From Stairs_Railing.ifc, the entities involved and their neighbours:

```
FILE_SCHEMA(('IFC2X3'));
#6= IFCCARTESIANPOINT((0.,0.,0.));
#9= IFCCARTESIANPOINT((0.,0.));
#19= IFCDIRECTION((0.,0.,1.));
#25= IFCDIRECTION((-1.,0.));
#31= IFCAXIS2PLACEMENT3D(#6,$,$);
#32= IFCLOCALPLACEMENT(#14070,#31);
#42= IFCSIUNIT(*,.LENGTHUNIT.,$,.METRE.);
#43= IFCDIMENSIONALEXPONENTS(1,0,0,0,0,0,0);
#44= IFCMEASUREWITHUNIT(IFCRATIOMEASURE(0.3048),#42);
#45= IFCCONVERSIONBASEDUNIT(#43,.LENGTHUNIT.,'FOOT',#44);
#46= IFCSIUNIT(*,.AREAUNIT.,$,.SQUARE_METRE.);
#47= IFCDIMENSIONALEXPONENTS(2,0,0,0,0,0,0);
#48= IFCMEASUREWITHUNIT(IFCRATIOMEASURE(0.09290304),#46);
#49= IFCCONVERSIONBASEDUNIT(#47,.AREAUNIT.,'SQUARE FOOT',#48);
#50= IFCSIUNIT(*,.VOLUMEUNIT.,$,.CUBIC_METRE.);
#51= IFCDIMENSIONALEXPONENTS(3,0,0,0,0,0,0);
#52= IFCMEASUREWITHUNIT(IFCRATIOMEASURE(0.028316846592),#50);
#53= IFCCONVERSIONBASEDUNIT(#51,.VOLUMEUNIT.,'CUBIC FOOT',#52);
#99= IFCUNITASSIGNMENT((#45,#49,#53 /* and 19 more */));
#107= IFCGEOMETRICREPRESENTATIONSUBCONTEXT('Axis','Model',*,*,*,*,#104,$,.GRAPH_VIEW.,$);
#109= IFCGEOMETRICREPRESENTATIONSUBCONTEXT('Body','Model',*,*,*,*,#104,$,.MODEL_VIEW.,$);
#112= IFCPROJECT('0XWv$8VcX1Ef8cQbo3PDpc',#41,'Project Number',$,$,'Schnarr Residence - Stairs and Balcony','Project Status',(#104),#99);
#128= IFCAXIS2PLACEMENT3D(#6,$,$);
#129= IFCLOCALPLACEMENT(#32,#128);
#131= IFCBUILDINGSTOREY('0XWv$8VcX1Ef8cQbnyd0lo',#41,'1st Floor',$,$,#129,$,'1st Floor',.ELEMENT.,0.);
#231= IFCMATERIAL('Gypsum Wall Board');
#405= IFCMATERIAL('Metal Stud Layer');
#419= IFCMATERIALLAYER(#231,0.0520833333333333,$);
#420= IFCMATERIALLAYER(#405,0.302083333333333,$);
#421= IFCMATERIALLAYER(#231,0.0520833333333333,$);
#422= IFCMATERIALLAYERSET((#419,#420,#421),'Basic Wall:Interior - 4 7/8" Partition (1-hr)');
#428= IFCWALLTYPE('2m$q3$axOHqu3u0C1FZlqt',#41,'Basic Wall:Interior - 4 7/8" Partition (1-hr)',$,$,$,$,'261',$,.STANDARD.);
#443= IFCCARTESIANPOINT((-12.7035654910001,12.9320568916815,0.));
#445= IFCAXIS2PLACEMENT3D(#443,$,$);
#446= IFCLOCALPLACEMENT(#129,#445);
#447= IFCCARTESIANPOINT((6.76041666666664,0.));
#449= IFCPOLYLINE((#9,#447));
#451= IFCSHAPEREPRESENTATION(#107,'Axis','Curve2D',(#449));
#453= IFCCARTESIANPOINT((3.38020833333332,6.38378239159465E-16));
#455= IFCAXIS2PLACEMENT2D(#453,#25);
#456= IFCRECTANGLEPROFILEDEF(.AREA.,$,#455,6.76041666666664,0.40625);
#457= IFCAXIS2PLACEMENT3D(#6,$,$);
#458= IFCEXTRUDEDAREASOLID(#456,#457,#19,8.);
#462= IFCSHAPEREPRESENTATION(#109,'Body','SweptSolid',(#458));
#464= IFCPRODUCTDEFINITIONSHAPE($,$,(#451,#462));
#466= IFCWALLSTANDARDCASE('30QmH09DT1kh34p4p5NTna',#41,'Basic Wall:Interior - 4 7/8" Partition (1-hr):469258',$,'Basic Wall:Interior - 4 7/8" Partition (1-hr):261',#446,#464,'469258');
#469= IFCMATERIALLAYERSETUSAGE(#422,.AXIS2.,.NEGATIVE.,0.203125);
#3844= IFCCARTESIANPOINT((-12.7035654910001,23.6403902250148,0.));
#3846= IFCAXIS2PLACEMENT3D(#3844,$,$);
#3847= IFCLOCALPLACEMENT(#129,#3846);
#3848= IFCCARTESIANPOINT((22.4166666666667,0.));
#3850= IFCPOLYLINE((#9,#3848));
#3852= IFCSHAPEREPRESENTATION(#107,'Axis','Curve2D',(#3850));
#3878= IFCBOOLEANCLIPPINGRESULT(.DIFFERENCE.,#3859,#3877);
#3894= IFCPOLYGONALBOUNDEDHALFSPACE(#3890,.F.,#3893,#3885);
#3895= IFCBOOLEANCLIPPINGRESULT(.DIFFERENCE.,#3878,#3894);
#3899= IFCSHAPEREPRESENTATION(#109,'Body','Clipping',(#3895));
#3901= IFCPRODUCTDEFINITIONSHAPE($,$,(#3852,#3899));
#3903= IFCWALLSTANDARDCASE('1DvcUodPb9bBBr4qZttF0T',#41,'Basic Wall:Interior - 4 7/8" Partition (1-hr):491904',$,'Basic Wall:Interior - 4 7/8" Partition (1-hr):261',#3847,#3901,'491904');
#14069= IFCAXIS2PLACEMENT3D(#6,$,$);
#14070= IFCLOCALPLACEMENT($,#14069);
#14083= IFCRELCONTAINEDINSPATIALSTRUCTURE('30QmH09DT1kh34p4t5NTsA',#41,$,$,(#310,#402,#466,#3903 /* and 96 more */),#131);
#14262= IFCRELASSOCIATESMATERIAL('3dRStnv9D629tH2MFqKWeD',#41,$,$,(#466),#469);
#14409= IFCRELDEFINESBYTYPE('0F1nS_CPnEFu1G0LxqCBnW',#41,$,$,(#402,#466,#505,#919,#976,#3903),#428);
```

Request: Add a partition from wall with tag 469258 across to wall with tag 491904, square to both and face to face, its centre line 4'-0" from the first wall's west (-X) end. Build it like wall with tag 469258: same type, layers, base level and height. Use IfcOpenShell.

```python
import numpy as np
import ifcopenshell
import ifcopenshell.api.geometry
import ifcopenshell.api.material
import ifcopenshell.api.pset
import ifcopenshell.api.root
import ifcopenshell.api.spatial
import ifcopenshell.api.type
import ifcopenshell.geom
import ifcopenshell.util.element
import ifcopenshell.util.placement
import ifcopenshell.util.representation
import ifcopenshell.util.shape
import ifcopenshell.util.unit

model = ifcopenshell.open("Stairs_Railing.ifc")
unit_scale = ifcopenshell.util.unit.calculate_unit_scale(model)
settings = ifcopenshell.geom.settings()
settings.set("use-world-coords", True)

start_wall = model.by_guid("30QmH09DT1kh34p4p5NTna")
end_wall = model.by_guid("1DvcUodPb9bBBr4qZttF0T")
like = model.by_id(466)
matrix = ifcopenshell.util.placement.get_local_placement(start_wall.ObjectPlacement)
matrix[:3, 3] *= unit_scale


def extent(element):
    """Bounding box in the first wall's axes, in metres."""
    shape = ifcopenshell.geom.create_shape(settings, element)
    points = (ifcopenshell.util.shape.get_vertices(shape.geometry) - matrix[:3, 3]) @ matrix[:3, :3]
    return points.min(axis=0), points.max(axis=0)


y_start = extent(start_wall)[1][1]
y_end = extent(end_wall)[0][1]
like_min, like_max = extent(like)
length, height = float(abs(y_end - y_start)), float(like_max[2] - like_min[2])
layer_set = ifcopenshell.util.element.get_material(like, should_skip_usage=True)
thickness = sum(layer.LayerThickness for layer in layer_set.MaterialLayers) * unit_scale

wall = ifcopenshell.api.root.create_entity(model, ifc_class="IfcWallStandardCase", name="New partition")
storey = ifcopenshell.util.element.get_container(like)
ifcopenshell.api.spatial.assign_container(model, products=[wall], relating_structure=storey)
ifcopenshell.api.type.assign_type(
    model, related_objects=[wall], relating_type=ifcopenshell.util.element.get_type(like), should_map_representations=False
)
rel = ifcopenshell.api.material.assign_material(
    model, products=[wall], type="IfcMaterialLayerSetUsage", material=layer_set
)
rel.RelatingMaterial.OffsetFromReferenceLine = -thickness / 2 / unit_scale
pset = ifcopenshell.api.pset.add_pset(model, product=wall, name="Pset_WallCommon")
ifcopenshell.api.pset.edit_pset(model, pset=pset, properties={"IsExternal": False, "LoadBearing": False})

# The axis runs down the middle of the wall.
axis = ifcopenshell.api.geometry.add_axis_representation(
    model, context=ifcopenshell.util.representation.get_context(model, "Model", "Axis"), axis=[(0.0, 0.0), (length, 0.0)]
)
body = ifcopenshell.api.geometry.add_wall_representation(
    model,
    context=ifcopenshell.util.representation.get_context(model, "Model", "Body", "MODEL_VIEW"),
    length=length,
    height=height,
    thickness=thickness,
    offset=-thickness / 2,
)
for representation in (axis, body):
    ifcopenshell.api.geometry.assign_representation(model, product=wall, representation=representation)

placement = matrix @ ifcopenshell.util.placement.rotation(90, "Z")
placement[:, 3] = matrix @ np.array([extent(start_wall)[0][0] + 1.2192, y_start, like_min[2], 1.0])
ifcopenshell.api.geometry.edit_object_placement(model, product=wall, matrix=placement)

print(f"partition {length:.3f} m long, {height:.3f} m high, {thickness:.3f} m thick")

model.write("Stairs_Railing_v2.ifc")
```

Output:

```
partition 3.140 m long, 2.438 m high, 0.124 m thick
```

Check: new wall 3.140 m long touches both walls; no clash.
